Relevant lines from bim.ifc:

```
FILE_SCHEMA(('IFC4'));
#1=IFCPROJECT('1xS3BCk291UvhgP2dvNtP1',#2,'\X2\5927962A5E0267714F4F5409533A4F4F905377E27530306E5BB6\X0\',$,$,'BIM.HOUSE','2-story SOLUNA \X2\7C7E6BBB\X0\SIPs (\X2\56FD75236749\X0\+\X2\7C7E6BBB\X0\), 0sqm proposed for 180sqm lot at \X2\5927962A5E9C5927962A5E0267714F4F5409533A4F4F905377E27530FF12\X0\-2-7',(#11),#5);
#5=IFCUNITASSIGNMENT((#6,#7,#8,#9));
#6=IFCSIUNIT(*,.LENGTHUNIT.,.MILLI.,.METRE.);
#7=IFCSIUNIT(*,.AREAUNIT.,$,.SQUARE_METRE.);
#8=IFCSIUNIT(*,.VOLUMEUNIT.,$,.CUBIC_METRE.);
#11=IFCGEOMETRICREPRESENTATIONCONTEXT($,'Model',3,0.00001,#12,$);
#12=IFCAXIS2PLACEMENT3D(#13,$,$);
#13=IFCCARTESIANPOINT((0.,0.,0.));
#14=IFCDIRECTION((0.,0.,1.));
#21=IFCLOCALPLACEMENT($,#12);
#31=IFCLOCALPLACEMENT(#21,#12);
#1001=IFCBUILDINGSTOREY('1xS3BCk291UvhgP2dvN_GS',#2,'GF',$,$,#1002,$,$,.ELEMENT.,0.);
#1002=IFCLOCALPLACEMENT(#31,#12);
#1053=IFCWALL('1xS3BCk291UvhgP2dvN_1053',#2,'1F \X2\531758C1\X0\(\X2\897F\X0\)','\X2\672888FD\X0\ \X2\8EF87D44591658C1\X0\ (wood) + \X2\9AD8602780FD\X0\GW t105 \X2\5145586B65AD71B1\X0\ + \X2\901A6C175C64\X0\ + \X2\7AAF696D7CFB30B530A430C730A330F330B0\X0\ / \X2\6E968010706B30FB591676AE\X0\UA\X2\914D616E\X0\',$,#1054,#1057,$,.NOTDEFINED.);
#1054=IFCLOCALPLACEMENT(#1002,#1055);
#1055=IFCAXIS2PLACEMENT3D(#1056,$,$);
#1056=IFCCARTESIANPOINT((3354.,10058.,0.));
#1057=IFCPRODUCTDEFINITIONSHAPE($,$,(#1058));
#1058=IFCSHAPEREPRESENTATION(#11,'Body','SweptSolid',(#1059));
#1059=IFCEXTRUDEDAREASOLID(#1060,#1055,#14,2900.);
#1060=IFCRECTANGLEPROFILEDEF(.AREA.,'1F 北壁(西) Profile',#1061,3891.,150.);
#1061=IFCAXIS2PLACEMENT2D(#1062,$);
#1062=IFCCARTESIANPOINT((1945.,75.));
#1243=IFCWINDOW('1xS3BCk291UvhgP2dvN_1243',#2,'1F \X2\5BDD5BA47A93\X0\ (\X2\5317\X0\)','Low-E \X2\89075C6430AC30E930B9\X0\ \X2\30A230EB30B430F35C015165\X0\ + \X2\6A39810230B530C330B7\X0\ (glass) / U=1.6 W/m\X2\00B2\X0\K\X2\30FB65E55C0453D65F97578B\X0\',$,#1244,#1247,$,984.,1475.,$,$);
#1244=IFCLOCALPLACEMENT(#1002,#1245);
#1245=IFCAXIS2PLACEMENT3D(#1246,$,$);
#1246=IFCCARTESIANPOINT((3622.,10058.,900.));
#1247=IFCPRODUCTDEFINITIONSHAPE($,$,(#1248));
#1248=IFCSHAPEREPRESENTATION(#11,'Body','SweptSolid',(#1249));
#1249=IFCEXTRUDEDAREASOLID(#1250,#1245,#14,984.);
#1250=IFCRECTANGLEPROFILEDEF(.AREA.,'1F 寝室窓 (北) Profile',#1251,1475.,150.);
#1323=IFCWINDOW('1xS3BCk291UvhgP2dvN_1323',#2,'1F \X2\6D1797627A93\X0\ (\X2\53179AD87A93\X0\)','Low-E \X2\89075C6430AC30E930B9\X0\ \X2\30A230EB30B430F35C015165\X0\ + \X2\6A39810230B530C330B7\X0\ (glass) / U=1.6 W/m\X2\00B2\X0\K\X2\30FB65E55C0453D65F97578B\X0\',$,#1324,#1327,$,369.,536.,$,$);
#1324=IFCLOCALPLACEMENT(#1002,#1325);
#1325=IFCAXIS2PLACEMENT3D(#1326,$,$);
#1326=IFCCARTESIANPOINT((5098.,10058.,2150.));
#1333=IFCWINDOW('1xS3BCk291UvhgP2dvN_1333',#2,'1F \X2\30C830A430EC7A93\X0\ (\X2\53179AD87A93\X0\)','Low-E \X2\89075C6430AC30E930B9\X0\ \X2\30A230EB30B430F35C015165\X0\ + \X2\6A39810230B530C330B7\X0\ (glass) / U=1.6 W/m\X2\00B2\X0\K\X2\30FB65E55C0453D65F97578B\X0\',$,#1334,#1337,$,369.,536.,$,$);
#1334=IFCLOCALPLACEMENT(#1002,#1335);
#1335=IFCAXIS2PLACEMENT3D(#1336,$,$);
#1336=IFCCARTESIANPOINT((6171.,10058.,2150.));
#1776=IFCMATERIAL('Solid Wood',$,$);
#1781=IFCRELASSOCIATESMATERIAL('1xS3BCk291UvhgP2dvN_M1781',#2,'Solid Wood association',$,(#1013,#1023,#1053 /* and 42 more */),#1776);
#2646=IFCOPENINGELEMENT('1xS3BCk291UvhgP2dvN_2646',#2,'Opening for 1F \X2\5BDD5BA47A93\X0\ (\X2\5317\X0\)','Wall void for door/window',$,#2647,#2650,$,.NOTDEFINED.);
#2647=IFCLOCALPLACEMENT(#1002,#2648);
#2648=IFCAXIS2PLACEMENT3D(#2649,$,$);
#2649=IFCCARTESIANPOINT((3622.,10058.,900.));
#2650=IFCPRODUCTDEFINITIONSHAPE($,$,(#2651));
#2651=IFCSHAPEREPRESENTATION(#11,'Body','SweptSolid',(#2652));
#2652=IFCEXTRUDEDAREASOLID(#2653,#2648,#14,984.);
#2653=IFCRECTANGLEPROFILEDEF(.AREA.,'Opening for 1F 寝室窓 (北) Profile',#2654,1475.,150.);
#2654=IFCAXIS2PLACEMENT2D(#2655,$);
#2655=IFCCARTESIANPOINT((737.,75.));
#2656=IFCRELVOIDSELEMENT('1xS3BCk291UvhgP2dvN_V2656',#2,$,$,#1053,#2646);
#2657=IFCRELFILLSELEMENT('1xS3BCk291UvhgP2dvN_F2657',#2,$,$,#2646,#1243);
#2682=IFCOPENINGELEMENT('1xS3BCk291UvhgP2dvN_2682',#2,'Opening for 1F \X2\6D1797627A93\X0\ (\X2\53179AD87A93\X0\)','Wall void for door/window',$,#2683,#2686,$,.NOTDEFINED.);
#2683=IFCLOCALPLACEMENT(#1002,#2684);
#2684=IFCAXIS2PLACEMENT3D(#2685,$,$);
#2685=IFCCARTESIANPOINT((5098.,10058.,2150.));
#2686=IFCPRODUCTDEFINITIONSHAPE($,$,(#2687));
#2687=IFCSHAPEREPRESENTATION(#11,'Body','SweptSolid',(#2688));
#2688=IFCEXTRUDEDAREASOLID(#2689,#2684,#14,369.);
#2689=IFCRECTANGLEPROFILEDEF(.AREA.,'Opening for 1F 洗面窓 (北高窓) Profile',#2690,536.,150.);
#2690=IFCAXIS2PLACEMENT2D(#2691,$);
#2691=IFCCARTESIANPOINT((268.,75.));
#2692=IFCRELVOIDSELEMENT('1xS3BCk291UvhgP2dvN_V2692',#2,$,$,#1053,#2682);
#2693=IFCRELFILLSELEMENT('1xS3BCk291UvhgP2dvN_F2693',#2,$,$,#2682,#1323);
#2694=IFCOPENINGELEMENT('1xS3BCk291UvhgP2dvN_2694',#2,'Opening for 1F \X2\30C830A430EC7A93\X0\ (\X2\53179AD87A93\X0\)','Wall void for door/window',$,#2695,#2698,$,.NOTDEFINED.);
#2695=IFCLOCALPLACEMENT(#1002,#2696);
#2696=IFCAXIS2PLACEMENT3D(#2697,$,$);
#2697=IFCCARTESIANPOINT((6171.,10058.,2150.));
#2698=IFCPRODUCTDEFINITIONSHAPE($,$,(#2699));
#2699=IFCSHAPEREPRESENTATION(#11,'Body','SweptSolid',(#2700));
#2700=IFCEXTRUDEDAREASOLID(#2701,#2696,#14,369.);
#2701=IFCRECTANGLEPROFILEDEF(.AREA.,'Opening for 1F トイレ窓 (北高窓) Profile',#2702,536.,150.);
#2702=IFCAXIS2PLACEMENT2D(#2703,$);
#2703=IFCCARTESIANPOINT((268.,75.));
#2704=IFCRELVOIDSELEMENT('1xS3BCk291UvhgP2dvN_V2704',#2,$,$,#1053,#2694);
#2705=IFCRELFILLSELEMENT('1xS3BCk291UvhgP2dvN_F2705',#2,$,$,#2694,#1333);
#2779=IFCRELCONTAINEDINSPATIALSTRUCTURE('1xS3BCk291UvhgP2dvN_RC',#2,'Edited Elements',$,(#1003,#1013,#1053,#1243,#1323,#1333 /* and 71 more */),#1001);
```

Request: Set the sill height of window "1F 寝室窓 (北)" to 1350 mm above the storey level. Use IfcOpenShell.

```python
import numpy as np
import ifcopenshell
import ifcopenshell.api.geometry
import ifcopenshell.geom
import ifcopenshell.util.element
import ifcopenshell.util.placement
import ifcopenshell.util.shape
import ifcopenshell.util.unit

model = ifcopenshell.open("bim.ifc")
unit_scale = ifcopenshell.util.unit.calculate_unit_scale(model)

window = model.by_guid("1xS3BCk291UvhgP2dvN_1243")
opening = window.FillsVoids[0].RelatingOpeningElement
storey = ifcopenshell.util.element.get_container(window, ifc_class="IfcBuildingStorey")
level = ifcopenshell.util.placement.get_local_placement(storey.ObjectPlacement)[2, 3]

# The opening's origin need not be at the sill, so measure its lowest point.
shape = ifcopenshell.geom.create_shape(ifcopenshell.geom.settings(), opening)
bottom = ifcopenshell.util.shape.get_shape_bottom_elevation(shape, shape.geometry) / unit_scale
dz = level + 1.35 / unit_scale - bottom

shift = np.array([0.0, 0.0, dz])
# The window is not placed relative to its opening, so move both.
for product in (opening, window):
    matrix = ifcopenshell.util.placement.get_local_placement(product.ObjectPlacement)
    matrix[:3, 3] += shift
    ifcopenshell.api.geometry.edit_object_placement(model, product=product, matrix=matrix, is_si=False)

print(f"moved by {dz * unit_scale:+.3f} m")

model.write("bim_edited.ifc")
```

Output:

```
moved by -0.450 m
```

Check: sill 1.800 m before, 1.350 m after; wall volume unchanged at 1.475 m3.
